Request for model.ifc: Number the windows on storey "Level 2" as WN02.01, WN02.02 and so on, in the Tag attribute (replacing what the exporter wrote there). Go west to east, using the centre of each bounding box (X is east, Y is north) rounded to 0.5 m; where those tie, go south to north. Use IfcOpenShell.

First a look at what the model holds.

```python
import ifcopenshell
import ifcopenshell.util.element
import ifcopenshell.util.placement

model = ifcopenshell.open("model.ifc")
print(model.schema)
storey = next(s for s in model.by_type("IfcBuildingStorey") if s.Name == "Level 2")
windows = [e for e in ifcopenshell.util.element.get_decomposition(storey) if e.is_a("IfcWindow")]
for e in sorted(windows, key=lambda e: e.id()):
    origin = ifcopenshell.util.placement.get_local_placement(e.ObjectPlacement)[:3, 3]
    print(e.id(), e.Tag, e.Name, origin.round(2) + 0.0, sep=" | ")
```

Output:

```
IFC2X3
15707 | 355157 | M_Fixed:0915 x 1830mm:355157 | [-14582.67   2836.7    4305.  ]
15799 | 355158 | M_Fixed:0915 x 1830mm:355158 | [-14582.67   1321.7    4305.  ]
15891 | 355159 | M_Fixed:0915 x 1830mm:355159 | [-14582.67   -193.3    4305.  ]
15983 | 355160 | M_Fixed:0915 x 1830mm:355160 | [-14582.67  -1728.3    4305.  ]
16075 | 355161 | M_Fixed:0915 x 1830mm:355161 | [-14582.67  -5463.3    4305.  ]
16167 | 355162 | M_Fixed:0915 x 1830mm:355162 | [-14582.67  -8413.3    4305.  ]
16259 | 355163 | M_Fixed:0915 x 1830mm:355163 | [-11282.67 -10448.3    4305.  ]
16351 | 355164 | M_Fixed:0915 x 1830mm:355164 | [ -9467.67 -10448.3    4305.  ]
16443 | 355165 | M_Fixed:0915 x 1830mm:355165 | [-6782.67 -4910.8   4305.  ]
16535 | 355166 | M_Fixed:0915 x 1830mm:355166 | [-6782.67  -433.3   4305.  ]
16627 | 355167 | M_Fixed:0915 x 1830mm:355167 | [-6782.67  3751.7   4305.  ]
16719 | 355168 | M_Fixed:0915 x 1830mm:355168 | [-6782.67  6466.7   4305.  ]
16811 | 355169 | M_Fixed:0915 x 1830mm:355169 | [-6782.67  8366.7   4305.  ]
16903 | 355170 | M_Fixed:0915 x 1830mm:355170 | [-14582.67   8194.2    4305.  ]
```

```python
import ifcopenshell
import ifcopenshell.geom
import ifcopenshell.util.element
import ifcopenshell.util.shape

model = ifcopenshell.open("model.ifc")
settings = ifcopenshell.geom.settings()
settings.set("use-world-coords", True)


def centre(element):
    shape = ifcopenshell.geom.create_shape(settings, element)
    return ifcopenshell.util.shape.get_bbox_centroid(shape.geometry)


storey = next(s for s in model.by_type("IfcBuildingStorey") if s.Name == "Level 2")
windows = [e for e in ifcopenshell.util.element.get_decomposition(storey) if e.is_a("IfcWindow")]

# Insertion points can sit at a corner or the storey origin, so sort by the geometry (in metres).
centres = {e: centre(e) for e in windows}
windows.sort(key=lambda e: (round(centres[e][0] / 0.5), centres[e][1]))

for i, e in enumerate(windows, start=1):
    number = f"WN02.{i:02d}"
    e.Tag = number
    print(e.id(), number)

model.write("model-out.ifc")
```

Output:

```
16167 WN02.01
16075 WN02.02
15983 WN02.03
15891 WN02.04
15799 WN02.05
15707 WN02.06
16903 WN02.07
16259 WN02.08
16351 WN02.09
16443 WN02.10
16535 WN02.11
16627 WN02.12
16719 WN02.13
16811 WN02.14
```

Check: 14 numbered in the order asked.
